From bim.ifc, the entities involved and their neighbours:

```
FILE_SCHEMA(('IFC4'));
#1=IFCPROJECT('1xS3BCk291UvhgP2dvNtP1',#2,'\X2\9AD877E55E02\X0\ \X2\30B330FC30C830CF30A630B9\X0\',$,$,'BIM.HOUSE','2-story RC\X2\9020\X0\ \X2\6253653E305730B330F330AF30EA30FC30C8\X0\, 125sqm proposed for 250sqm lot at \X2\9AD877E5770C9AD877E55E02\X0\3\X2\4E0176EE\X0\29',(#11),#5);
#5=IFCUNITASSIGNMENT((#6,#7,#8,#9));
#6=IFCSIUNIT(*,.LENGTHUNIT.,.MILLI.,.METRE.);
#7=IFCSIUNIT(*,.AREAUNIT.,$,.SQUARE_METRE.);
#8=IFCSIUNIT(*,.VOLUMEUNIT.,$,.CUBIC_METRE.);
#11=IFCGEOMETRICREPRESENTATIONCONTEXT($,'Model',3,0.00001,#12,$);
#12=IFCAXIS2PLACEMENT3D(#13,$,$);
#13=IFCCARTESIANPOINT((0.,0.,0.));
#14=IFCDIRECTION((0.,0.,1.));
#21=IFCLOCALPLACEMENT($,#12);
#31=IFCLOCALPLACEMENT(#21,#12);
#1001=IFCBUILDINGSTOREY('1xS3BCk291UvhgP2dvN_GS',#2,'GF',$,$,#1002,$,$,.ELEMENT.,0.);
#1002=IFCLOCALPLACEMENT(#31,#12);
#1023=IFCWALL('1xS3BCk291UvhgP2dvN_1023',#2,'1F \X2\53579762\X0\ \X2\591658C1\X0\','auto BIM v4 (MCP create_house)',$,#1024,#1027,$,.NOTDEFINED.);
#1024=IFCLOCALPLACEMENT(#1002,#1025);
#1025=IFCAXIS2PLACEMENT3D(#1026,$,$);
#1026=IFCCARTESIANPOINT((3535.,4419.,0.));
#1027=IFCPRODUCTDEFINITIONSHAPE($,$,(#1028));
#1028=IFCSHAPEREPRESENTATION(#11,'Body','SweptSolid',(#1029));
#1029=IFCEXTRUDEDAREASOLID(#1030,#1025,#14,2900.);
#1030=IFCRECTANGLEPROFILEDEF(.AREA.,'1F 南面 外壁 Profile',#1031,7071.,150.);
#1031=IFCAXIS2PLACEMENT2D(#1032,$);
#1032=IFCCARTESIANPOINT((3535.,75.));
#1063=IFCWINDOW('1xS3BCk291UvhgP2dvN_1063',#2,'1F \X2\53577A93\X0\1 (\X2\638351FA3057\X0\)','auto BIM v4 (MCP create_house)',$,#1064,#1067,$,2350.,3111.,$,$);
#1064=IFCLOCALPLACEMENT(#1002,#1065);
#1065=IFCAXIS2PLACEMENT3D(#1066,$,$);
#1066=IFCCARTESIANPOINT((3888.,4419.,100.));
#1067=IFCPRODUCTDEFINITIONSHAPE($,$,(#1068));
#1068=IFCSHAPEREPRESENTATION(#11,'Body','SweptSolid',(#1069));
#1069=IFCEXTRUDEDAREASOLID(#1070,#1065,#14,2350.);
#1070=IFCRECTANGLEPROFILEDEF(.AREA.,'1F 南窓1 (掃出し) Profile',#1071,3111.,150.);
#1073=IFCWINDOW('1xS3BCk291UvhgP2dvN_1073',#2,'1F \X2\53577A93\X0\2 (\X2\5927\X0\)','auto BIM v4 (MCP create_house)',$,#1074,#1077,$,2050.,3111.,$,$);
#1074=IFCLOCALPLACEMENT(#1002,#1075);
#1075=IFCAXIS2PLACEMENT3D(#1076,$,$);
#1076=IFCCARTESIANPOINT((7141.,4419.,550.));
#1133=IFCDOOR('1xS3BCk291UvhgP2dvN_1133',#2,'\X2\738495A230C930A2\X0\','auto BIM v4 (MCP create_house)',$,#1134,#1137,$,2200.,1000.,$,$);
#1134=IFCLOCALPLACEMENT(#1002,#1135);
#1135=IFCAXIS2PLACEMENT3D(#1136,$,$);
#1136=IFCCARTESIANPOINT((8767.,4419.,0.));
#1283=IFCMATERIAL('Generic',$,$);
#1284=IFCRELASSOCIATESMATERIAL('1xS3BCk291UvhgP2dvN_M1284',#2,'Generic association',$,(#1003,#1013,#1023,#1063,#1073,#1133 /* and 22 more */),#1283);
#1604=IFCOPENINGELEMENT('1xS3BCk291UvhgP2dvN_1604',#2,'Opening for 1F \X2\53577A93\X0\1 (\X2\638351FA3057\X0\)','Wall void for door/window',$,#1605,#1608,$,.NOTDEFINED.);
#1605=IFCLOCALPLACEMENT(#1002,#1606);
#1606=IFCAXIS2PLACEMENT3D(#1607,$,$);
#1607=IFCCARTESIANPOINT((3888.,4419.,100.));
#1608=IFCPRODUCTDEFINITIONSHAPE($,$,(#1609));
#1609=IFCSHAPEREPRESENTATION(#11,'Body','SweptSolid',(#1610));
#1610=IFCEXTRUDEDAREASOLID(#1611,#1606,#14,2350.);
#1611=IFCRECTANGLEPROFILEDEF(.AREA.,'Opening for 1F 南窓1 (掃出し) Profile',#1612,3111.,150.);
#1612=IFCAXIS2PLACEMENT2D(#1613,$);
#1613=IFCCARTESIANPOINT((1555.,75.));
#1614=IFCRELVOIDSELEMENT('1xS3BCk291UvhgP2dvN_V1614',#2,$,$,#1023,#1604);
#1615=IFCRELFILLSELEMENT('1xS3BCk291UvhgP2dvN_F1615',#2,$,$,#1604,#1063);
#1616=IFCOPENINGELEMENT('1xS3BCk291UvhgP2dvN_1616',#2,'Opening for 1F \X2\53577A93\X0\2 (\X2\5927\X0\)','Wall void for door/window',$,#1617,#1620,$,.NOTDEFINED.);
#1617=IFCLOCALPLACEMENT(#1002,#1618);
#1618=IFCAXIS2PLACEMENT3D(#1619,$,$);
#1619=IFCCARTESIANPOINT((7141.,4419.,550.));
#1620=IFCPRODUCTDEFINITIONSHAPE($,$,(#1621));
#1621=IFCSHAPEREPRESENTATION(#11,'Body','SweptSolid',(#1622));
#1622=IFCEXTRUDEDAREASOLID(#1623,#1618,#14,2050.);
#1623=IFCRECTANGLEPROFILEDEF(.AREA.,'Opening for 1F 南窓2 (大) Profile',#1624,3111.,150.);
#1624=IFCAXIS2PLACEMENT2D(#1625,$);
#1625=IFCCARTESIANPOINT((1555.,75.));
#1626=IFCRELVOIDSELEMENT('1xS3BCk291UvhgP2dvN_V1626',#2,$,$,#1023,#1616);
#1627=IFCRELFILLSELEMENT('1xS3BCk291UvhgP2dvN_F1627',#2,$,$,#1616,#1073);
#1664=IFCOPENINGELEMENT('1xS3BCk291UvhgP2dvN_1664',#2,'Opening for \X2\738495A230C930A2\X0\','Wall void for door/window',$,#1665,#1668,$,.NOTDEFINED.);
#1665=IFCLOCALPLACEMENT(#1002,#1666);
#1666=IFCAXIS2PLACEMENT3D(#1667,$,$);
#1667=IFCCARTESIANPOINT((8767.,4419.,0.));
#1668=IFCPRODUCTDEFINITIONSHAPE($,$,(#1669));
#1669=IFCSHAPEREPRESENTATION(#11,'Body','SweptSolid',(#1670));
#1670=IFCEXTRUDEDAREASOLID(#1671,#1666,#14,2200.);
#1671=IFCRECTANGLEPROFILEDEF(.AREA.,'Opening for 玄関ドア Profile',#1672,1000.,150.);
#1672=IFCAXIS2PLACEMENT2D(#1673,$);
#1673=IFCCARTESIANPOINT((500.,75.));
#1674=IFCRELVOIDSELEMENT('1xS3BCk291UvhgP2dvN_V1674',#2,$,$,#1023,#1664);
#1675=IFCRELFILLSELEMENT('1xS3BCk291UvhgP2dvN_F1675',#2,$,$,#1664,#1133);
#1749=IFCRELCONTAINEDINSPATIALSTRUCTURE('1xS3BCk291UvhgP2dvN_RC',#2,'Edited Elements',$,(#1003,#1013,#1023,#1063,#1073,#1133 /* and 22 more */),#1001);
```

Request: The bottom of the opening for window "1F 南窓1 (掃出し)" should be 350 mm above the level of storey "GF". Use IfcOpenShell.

```python
import numpy as np
import ifcopenshell
import ifcopenshell.api.geometry
import ifcopenshell.geom
import ifcopenshell.util.element
import ifcopenshell.util.placement
import ifcopenshell.util.shape
import ifcopenshell.util.unit

model = ifcopenshell.open("bim.ifc")
unit_scale = ifcopenshell.util.unit.calculate_unit_scale(model)

window = model.by_id(1063)
opening = window.FillsVoids[0].RelatingOpeningElement
storey = ifcopenshell.util.element.get_container(window, ifc_class="IfcBuildingStorey")
level = ifcopenshell.util.placement.get_local_placement(storey.ObjectPlacement)[2, 3]

# The opening's origin need not be at the sill, so measure its lowest point.
shape = ifcopenshell.geom.create_shape(ifcopenshell.geom.settings(), opening)
bottom = ifcopenshell.util.shape.get_shape_bottom_elevation(shape, shape.geometry) / unit_scale
dz = level + 0.35 / unit_scale - bottom

shift = np.array([0.0, 0.0, dz])
# The window is not placed relative to its opening, so move both.
for product in (opening, window):
    matrix = ifcopenshell.util.placement.get_local_placement(product.ObjectPlacement)
    matrix[:3, 3] += shift
    ifcopenshell.api.geometry.edit_object_placement(model, product=product, matrix=matrix, is_si=False)

print(f"moved by {dz * unit_scale:+.3f} m")

model.write("bim_rev.ifc")
```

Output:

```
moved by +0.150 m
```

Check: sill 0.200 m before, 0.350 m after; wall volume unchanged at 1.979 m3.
